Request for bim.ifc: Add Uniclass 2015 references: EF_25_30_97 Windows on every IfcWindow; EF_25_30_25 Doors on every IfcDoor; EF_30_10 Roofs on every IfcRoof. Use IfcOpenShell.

First a look at what the model holds.

```python
import ifcopenshell

model = ifcopenshell.open("bim.ifc")
print(model.schema)
print("classifications:", [c.Name for c in model.by_type("IfcClassification")])
for ifc_class in ("IfcDoor", "IfcRoof", "IfcStair", "IfcWall", "IfcWindow"):
    print(ifc_class, len(model.by_type(ifc_class)))
```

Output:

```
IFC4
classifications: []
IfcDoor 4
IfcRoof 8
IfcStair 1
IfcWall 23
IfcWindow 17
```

```python
import ifcopenshell
import ifcopenshell.api.classification

model = ifcopenshell.open("bim.ifc")

system = ifcopenshell.api.classification.add_classification(model, classification="Uniclass 2015")

codes = {
    "IfcWindow": ("EF_25_30_97", "Windows"),
    "IfcDoor": ("EF_25_30_25", "Doors"),
    "IfcRoof": ("EF_30_10", "Roofs"),
}
for ifc_class, (code, name) in codes.items():
    products = model.by_type(ifc_class)
    ifcopenshell.api.classification.add_reference(
        model, products=products, classification=system, identification=code, name=name
    )
    print(code, len(products))

model.write("bim_updated.ifc")
```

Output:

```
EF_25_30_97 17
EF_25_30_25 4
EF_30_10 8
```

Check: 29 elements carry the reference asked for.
